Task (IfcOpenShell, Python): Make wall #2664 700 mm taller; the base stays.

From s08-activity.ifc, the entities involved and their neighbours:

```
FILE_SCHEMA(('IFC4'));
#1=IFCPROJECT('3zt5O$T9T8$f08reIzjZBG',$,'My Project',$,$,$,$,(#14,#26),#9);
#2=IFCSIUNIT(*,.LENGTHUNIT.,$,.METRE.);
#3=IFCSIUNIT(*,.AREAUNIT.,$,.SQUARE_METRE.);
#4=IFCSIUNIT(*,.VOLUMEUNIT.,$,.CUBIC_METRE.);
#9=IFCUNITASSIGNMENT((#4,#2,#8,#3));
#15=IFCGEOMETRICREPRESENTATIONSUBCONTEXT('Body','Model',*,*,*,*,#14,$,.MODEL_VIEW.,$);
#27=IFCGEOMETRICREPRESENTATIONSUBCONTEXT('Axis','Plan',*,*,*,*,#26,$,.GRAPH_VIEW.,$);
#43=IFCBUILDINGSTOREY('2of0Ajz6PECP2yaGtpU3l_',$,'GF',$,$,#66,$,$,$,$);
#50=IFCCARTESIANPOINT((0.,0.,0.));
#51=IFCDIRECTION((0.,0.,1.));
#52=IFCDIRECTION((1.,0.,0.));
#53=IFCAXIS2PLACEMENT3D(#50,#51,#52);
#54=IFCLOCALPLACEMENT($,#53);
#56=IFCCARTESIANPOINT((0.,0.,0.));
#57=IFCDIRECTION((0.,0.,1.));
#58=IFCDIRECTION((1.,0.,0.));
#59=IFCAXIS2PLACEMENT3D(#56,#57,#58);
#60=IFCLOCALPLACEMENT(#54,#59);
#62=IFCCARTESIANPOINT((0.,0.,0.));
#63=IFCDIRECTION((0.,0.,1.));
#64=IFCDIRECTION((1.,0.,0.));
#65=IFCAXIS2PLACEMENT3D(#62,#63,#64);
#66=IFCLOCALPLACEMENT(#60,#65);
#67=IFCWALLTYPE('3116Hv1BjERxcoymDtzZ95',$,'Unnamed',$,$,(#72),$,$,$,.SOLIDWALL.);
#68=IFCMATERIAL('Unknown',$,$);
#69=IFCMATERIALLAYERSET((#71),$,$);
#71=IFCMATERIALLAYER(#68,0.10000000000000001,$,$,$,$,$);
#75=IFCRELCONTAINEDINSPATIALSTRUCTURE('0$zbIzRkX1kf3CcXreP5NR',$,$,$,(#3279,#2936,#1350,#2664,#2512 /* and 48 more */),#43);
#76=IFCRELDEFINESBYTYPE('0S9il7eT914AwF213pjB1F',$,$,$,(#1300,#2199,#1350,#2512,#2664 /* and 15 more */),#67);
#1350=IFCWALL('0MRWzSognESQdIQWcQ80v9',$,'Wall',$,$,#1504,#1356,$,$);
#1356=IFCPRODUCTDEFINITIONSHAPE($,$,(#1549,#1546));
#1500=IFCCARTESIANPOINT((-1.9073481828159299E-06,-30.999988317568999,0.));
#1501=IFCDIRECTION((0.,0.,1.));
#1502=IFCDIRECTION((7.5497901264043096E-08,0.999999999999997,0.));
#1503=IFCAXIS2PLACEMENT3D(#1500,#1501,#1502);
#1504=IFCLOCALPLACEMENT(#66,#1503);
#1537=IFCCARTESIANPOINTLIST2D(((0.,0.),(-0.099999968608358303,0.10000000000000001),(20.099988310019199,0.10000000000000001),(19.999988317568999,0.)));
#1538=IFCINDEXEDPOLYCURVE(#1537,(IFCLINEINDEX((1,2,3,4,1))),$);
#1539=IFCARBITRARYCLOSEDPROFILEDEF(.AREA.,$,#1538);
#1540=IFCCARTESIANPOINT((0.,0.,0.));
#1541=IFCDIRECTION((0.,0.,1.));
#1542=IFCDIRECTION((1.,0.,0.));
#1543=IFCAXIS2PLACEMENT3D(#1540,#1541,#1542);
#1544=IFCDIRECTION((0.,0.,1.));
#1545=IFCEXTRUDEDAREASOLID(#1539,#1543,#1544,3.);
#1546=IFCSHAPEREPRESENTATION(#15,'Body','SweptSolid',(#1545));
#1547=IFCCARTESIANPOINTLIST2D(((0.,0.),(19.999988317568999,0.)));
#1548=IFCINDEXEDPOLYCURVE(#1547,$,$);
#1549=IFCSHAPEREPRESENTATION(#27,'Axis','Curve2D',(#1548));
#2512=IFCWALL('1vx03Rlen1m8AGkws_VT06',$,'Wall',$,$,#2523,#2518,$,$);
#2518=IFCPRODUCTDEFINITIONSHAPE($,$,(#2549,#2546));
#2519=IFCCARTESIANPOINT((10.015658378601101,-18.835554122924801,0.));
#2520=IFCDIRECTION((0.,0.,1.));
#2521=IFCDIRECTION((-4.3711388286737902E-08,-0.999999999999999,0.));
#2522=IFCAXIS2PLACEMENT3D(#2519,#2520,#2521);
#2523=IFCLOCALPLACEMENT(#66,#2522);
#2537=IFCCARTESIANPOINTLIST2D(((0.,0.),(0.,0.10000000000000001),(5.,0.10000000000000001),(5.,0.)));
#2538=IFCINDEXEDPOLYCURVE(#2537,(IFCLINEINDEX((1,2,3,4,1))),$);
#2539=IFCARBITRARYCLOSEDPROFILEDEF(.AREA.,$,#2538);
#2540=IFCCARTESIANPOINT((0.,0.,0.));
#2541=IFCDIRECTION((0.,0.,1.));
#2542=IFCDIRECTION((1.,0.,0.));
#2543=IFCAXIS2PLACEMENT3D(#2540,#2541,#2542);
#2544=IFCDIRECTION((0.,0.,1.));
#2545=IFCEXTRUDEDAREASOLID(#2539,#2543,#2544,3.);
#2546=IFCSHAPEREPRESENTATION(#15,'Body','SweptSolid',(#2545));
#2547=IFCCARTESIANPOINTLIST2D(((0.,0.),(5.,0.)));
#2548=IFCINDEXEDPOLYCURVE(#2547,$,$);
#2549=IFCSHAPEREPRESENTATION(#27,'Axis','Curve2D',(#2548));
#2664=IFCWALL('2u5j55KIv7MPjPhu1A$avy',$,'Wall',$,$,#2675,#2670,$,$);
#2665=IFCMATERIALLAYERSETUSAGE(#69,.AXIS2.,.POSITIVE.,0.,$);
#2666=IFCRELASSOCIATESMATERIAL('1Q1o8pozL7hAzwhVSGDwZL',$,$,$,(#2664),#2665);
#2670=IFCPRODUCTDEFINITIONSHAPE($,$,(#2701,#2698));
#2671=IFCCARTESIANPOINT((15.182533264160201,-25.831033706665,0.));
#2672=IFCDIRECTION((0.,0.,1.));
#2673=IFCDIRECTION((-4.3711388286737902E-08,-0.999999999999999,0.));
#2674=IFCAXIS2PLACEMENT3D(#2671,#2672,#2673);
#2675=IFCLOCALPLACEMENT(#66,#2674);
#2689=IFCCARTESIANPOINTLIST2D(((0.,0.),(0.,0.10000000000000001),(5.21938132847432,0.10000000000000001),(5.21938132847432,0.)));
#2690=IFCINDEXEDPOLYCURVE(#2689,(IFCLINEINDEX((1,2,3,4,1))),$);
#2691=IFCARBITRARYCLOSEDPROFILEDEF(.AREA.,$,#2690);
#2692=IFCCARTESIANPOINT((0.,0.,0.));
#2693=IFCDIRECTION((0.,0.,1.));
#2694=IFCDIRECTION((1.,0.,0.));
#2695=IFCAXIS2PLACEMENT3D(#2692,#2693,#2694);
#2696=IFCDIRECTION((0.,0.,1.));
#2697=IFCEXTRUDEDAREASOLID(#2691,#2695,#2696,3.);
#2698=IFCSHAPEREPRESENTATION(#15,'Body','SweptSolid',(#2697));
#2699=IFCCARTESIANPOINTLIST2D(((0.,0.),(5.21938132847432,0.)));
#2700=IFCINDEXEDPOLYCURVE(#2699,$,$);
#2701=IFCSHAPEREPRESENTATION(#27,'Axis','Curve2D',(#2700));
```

```python
import ifcopenshell
import ifcopenshell.geom
import ifcopenshell.util.representation
import ifcopenshell.util.shape
import ifcopenshell.util.unit

model = ifcopenshell.open("s08-activity.ifc")
unit_scale = ifcopenshell.util.unit.calculate_unit_scale(model)
settings = ifcopenshell.geom.settings()


def volume(element):
    """Net volume in cubic metres, openings subtracted."""
    shape = ifcopenshell.geom.create_shape(settings, element)
    return ifcopenshell.util.shape.get_volume(shape.geometry)


wall = model.by_guid("2u5j55KIv7MPjPhu1A$avy")
before = volume(wall)

body = ifcopenshell.util.representation.get_representation(wall, "Model", "Body")
solid = body.Items[0]
old_height = solid.Depth
solid.Depth += 0.7 / unit_scale
after = volume(wall)

print(f"height {old_height:g} -> {solid.Depth:g}, volume {before:.3f} -> {after:.3f} m3")

model.write("s08-activity_updated.ifc")
```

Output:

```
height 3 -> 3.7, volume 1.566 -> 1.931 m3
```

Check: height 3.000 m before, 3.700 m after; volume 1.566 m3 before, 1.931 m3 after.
